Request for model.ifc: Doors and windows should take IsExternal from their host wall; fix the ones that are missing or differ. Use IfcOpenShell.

First a look at what the model holds.

```python
import ifcopenshell
import ifcopenshell.util.element

model = ifcopenshell.open("model.ifc")
print(model.schema)
seen = {}
for e in model.by_type("IfcDoor") + model.by_type("IfcWindow"):
    if not e.FillsVoids:
        continue
    host = e.FillsVoids[0].RelatingOpeningElement.VoidsElements[0].RelatingBuildingElement
    own = ifcopenshell.util.element.get_pset(e, f"Pset_{e.is_a()[3:].removesuffix('StandardCase')}Common", "IsExternal")
    wall = ifcopenshell.util.element.get_pset(host, "Pset_WallCommon", "IsExternal")
    seen[e.is_a(), own, wall] = seen.get((e.is_a(), own, wall), 0) + 1
for (cls, own, wall), count in sorted(seen.items(), key=str):
    print(count, cls, "IsExternal:", own, "| host wall:", wall)
```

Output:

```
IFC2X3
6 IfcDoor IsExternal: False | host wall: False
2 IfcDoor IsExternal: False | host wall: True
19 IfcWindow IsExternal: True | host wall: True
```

```python
import ifcopenshell
import ifcopenshell.api.pset
import ifcopenshell.util.element

model = ifcopenshell.open("model.ifc")

count = 0
for ifc_class, pset_name in (("IfcDoor", "Pset_DoorCommon"), ("IfcWindow", "Pset_WindowCommon")):
    for e in model.by_type(ifc_class):
        if not e.FillsVoids:
            continue
        host = e.FillsVoids[0].RelatingOpeningElement.VoidsElements[0].RelatingBuildingElement
        external = ifcopenshell.util.element.get_pset(host, "Pset_WallCommon", "IsExternal")
        if external is None or ifcopenshell.util.element.get_pset(e, pset_name, "IsExternal") == external:
            continue
        pset = ifcopenshell.api.pset.add_pset(model, product=e, name=pset_name)
        ifcopenshell.api.pset.edit_pset(model, pset=pset, properties={"IsExternal": external})
        count += 1

print(count, "updated")

model.write("model_v2.ifc")
```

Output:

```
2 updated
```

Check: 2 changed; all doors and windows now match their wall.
